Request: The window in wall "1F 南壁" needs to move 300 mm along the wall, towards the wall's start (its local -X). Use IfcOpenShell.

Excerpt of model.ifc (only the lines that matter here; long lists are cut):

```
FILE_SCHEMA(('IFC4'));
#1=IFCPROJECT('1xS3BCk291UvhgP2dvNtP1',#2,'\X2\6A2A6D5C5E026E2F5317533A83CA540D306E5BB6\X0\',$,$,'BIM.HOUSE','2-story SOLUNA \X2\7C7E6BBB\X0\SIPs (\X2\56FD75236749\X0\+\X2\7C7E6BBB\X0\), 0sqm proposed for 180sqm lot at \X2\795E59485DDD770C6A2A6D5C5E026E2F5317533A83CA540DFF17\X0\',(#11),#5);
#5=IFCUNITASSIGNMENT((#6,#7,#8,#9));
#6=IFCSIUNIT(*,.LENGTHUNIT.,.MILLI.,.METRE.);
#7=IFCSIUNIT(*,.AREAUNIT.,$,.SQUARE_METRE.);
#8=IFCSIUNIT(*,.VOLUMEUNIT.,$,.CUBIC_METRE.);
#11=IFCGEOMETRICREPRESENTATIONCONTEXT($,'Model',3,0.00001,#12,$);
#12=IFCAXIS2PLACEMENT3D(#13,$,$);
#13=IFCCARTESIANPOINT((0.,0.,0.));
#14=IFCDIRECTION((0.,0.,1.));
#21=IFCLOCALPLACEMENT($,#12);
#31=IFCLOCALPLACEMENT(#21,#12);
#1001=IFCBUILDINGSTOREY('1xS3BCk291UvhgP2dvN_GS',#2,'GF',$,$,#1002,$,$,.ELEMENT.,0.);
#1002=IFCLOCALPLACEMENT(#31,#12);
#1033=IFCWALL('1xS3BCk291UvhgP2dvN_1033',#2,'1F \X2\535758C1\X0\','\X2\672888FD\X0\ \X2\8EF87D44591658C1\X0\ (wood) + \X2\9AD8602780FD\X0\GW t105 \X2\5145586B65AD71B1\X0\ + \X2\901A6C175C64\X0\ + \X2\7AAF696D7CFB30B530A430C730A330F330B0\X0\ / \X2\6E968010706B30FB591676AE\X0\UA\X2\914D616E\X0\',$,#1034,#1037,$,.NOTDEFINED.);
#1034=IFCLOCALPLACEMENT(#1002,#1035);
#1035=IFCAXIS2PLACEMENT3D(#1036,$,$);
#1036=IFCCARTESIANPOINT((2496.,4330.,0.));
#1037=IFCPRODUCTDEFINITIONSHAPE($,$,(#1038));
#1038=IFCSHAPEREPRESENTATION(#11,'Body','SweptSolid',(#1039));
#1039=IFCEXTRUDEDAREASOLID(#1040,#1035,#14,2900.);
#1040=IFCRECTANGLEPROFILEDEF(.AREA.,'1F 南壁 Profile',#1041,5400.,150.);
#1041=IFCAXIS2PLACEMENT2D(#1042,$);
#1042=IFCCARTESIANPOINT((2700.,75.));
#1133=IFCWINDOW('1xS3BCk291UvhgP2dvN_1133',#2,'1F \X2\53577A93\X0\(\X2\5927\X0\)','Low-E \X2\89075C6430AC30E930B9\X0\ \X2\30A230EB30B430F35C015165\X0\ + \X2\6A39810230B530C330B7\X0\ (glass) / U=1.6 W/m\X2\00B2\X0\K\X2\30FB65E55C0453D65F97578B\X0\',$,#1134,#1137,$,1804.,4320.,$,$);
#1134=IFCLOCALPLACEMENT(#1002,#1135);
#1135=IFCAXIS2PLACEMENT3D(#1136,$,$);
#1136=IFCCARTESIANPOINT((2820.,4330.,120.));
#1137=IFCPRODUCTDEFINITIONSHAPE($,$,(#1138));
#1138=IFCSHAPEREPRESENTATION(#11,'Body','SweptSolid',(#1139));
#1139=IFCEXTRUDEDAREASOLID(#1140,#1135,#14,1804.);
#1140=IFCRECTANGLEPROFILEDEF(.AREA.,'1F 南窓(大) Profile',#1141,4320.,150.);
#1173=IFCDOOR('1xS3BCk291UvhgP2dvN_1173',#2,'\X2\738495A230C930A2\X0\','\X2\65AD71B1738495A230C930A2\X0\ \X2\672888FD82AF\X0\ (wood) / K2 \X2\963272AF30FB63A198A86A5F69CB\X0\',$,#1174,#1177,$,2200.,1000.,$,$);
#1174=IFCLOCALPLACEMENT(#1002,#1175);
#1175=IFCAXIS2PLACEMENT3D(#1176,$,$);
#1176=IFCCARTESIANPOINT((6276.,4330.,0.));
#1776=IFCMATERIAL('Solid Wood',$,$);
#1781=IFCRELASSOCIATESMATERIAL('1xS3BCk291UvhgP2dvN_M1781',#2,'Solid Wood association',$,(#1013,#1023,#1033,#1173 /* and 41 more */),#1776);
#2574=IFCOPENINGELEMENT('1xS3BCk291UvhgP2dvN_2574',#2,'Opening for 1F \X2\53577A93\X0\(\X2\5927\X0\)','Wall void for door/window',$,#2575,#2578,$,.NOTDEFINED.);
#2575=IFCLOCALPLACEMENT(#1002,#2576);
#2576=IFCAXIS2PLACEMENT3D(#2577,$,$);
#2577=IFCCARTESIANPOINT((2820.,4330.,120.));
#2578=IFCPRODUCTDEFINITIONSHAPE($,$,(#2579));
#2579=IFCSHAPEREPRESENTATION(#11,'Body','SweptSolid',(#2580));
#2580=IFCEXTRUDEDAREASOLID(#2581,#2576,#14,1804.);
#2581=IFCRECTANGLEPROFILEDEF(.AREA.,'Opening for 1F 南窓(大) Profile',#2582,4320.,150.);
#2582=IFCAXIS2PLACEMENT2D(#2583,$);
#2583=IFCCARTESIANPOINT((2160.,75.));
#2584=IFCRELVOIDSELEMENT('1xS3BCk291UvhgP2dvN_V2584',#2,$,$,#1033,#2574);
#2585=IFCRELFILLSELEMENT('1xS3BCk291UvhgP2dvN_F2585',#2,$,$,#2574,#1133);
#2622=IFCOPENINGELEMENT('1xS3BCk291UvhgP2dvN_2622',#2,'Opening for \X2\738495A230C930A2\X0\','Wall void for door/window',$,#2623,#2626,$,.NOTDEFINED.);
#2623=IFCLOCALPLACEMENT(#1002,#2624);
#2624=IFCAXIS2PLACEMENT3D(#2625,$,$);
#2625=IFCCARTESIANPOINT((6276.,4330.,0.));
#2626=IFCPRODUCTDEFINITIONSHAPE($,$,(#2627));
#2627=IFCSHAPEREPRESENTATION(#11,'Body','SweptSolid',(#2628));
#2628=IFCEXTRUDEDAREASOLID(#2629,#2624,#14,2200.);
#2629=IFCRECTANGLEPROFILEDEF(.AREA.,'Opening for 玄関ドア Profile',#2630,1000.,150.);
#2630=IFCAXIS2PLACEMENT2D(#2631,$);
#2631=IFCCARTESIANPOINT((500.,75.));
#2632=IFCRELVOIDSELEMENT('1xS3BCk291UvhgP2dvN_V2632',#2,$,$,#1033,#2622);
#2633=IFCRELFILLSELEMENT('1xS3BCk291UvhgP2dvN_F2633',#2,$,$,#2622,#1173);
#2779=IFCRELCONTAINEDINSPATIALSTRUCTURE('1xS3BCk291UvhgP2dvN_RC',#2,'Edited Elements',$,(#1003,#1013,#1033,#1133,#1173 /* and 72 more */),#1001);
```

```python
import ifcopenshell
import ifcopenshell.api.geometry
import ifcopenshell.util.placement

model = ifcopenshell.open("model.ifc")

window = model.by_guid("1xS3BCk291UvhgP2dvN_1133")
opening = window.FillsVoids[0].RelatingOpeningElement
wall = opening.VoidsElements[0].RelatingBuildingElement

wall_matrix = ifcopenshell.util.placement.get_local_placement(wall.ObjectPlacement)
shift = wall_matrix[:3, 0] * -300.0
before = ifcopenshell.util.placement.get_local_placement(window.ObjectPlacement)[:3, 3].copy()

# The window is not placed relative to its opening, so move both.
for product in (opening, window):
    matrix = ifcopenshell.util.placement.get_local_placement(product.ObjectPlacement)
    matrix[:3, 3] += shift
    ifcopenshell.api.geometry.edit_object_placement(model, product=product, matrix=matrix, is_si=False)

after = ifcopenshell.util.placement.get_local_placement(window.ObjectPlacement)[:3, 3]
print("window moved by", (after - before).round(3) + 0.0)

model.write("model_edited.ifc")
```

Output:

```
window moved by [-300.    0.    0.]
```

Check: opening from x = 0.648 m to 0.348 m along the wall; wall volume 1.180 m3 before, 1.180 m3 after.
